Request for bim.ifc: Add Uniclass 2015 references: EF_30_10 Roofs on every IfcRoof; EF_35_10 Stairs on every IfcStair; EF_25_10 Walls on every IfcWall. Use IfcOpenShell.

First a look at what the model holds.

```python
import ifcopenshell

model = ifcopenshell.open("bim.ifc")
print(model.schema)
print("classifications:", [c.Name for c in model.by_type("IfcClassification")])
for ifc_class in ("IfcDoor", "IfcRoof", "IfcStair", "IfcWall", "IfcWindow"):
    print(ifc_class, len(model.by_type(ifc_class)))
```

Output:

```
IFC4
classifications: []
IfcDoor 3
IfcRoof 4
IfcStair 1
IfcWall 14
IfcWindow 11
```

```python
import ifcopenshell
import ifcopenshell.api.classification

model = ifcopenshell.open("bim.ifc")

system = ifcopenshell.api.classification.add_classification(model, classification="Uniclass 2015")

codes = {
    "IfcRoof": ("EF_30_10", "Roofs"),
    "IfcStair": ("EF_35_10", "Stairs"),
    "IfcWall": ("EF_25_10", "Walls"),
}
for ifc_class, (code, name) in codes.items():
    products = model.by_type(ifc_class)
    ifcopenshell.api.classification.add_reference(
        model, products=products, classification=system, identification=code, name=name
    )
    print(code, len(products))

model.write("bim_rev.ifc")
```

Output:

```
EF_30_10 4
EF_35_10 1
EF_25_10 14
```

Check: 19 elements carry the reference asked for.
